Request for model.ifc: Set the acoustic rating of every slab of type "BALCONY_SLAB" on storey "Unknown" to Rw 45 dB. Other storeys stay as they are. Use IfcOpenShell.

First a look at what the model holds.

```python
import ifcopenshell
import ifcopenshell.util.element

model = ifcopenshell.open("model.ifc")
print(model.schema)
storey = next(s for s in model.by_type("IfcBuildingStorey") if s.Name == "Unknown")
slabs = [e for e in ifcopenshell.util.element.get_decomposition(storey) if e.is_a("IfcSlab")]
seen = {}
for e in slabs:
    element_type = ifcopenshell.util.element.get_type(e)
    key = (element_type.Name if element_type != e and element_type else None, ifcopenshell.util.element.get_pset(e, "Pset_SlabCommon", "AcousticRating"))
    seen[key] = seen.get(key, 0) + 1
for (name, value), count in sorted(seen.items(), key=str):
    print(count, "x", name, "|", value)
```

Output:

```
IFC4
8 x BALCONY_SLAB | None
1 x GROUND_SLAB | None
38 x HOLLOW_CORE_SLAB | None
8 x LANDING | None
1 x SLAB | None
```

```python
import ifcopenshell
import ifcopenshell.api.pset
import ifcopenshell.util.element

model = ifcopenshell.open("model.ifc")

storey = next(s for s in model.by_type("IfcBuildingStorey") if s.Name == "Unknown")
slabs = [e for e in ifcopenshell.util.element.get_decomposition(storey) if e.is_a("IfcSlab")]

count = 0
for e in slabs:
    element_type = ifcopenshell.util.element.get_type(e)
    if element_type in (None, e) or element_type.Name != "BALCONY_SLAB":
        continue
    found = ifcopenshell.util.element.get_pset(e, "Pset_SlabCommon", should_inherit=False)
    if found:
        pset = model.by_id(found["id"])
        if len(ifcopenshell.util.element.get_elements_by_pset(pset)) > 1:
            pset = ifcopenshell.api.pset.unshare_pset(model, products=[e], pset=pset)[0]
    else:
        pset = ifcopenshell.api.pset.add_pset(model, product=e, name="Pset_SlabCommon")
    ifcopenshell.api.pset.edit_pset(model, pset=pset, properties={"AcousticRating": "Rw 45 dB"})
    count += 1

print(count, "slabs updated")

model.write("model_v2.ifc")
```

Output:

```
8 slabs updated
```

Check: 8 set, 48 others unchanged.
